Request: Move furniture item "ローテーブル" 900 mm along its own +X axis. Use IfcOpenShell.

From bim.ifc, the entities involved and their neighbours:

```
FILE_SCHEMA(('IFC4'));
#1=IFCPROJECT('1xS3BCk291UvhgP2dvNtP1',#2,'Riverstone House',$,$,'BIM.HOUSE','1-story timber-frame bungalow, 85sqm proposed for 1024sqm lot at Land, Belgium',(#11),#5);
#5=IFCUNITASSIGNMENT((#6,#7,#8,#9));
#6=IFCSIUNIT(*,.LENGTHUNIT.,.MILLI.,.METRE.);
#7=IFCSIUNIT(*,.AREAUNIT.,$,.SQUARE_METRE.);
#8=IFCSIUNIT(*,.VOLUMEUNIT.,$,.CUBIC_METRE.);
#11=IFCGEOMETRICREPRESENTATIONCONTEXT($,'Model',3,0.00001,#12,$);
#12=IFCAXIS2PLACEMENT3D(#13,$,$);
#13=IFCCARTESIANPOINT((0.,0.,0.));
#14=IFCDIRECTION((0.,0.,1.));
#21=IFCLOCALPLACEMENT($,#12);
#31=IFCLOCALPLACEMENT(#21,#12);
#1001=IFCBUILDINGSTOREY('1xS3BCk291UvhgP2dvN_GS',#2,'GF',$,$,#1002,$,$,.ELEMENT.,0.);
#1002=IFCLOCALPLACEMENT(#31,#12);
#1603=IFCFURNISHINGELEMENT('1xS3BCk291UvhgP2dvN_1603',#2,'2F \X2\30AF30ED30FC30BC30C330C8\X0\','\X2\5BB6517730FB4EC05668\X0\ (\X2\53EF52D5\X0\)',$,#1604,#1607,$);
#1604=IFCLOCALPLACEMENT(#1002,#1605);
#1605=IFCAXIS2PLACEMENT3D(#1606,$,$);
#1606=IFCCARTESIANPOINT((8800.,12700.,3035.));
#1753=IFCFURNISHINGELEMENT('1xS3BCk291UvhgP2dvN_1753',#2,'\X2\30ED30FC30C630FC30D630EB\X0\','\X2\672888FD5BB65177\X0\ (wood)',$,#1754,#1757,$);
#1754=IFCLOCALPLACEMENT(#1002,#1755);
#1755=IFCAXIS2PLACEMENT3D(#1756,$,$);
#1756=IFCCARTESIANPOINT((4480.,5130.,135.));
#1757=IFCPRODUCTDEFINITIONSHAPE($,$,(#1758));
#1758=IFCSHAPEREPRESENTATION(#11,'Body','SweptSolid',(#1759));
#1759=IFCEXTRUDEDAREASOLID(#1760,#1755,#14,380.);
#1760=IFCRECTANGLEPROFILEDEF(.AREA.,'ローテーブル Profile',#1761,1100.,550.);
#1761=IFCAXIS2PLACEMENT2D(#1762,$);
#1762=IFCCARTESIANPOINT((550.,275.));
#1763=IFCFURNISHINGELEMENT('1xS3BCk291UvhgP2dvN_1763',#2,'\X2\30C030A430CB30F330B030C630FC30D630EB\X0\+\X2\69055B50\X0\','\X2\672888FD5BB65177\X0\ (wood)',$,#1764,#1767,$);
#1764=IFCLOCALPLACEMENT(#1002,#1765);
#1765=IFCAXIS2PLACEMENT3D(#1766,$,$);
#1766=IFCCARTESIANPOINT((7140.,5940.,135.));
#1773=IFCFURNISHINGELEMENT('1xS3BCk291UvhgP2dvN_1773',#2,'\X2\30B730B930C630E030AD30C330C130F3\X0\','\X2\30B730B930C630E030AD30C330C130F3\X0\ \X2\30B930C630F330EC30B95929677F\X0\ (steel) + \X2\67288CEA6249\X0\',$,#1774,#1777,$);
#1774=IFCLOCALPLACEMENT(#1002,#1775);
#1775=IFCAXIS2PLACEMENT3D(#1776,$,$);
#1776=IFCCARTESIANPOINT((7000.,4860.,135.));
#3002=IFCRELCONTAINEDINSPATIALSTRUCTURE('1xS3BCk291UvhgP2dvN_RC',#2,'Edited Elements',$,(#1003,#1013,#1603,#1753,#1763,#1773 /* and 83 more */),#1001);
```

```python
import ifcopenshell
import ifcopenshell.api.geometry
import ifcopenshell.util.placement
import ifcopenshell.util.unit

model = ifcopenshell.open("bim.ifc")
unit_scale = ifcopenshell.util.unit.calculate_unit_scale(model)

item = model.by_id(1753)
matrix = ifcopenshell.util.placement.get_local_placement(item.ObjectPlacement)
matrix[:3, 3] += matrix[:3, 0] * 0.9 / unit_scale
ifcopenshell.api.geometry.edit_object_placement(model, product=item, matrix=matrix, is_si=False)

print(ifcopenshell.util.placement.get_local_placement(item.ObjectPlacement).round(3) + 0.0)

model.write("bim-out.ifc")
```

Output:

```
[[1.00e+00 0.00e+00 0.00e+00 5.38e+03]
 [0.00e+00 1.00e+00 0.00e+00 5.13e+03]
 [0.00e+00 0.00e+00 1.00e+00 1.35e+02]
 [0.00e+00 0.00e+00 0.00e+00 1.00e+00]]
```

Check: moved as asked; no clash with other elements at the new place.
